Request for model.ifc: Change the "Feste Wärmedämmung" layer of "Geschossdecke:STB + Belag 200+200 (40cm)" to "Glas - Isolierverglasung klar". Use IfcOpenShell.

First a look at what the model holds.

```python
import ifcopenshell
import ifcopenshell.util.element

model = ifcopenshell.open("model.ifc")
print(model.schema)
for layer_set in model.by_type("IfcMaterialLayerSet"):
    if layer_set.LayerSetName == "Geschossdecke:STB + Belag 200+200 (40cm)":
        for layer in layer_set.MaterialLayers:
            print(layer.id(), layer.Material and layer.Material.Name, layer.LayerThickness, sep=" | ")
        print(len(ifcopenshell.util.element.get_elements_by_material(model, layer_set)), "elements and types use it")
print(sorted(m.Name for m in model.by_type("IfcMaterial") if m.Name)[:60])
```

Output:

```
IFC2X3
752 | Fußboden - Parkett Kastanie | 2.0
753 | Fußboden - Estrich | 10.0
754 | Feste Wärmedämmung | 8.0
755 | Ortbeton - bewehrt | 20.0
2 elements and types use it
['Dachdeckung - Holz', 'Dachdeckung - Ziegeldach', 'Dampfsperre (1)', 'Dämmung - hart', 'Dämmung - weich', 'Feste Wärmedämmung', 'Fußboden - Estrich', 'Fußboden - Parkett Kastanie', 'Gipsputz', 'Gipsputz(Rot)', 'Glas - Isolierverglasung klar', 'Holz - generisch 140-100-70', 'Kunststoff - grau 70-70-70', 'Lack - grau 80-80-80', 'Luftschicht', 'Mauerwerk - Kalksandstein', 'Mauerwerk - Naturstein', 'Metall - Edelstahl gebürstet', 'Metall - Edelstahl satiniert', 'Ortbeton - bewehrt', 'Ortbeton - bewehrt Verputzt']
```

```python
import ifcopenshell
import ifcopenshell.api.material

model = ifcopenshell.open("model.ifc")

layer_set = next(s for s in model.by_type("IfcMaterialLayerSet") if s.LayerSetName == "Geschossdecke:STB + Belag 200+200 (40cm)")
layer = next(l for l in layer_set.MaterialLayers if l.Material and l.Material.Name == "Feste Wärmedämmung")
material = next(m for m in model.by_type("IfcMaterial") if m.Name == "Glas - Isolierverglasung klar")

# Point this one layer at the other material; renaming the old one would change it everywhere.
ifcopenshell.api.material.edit_layer(model, layer=layer, attributes={}, material=material)

print([l.Material.Name if l.Material else None for l in layer_set.MaterialLayers])

model.write("model_v2.ifc")
```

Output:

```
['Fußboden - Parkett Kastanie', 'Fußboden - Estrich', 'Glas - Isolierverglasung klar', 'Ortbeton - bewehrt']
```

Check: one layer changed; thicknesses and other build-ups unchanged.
